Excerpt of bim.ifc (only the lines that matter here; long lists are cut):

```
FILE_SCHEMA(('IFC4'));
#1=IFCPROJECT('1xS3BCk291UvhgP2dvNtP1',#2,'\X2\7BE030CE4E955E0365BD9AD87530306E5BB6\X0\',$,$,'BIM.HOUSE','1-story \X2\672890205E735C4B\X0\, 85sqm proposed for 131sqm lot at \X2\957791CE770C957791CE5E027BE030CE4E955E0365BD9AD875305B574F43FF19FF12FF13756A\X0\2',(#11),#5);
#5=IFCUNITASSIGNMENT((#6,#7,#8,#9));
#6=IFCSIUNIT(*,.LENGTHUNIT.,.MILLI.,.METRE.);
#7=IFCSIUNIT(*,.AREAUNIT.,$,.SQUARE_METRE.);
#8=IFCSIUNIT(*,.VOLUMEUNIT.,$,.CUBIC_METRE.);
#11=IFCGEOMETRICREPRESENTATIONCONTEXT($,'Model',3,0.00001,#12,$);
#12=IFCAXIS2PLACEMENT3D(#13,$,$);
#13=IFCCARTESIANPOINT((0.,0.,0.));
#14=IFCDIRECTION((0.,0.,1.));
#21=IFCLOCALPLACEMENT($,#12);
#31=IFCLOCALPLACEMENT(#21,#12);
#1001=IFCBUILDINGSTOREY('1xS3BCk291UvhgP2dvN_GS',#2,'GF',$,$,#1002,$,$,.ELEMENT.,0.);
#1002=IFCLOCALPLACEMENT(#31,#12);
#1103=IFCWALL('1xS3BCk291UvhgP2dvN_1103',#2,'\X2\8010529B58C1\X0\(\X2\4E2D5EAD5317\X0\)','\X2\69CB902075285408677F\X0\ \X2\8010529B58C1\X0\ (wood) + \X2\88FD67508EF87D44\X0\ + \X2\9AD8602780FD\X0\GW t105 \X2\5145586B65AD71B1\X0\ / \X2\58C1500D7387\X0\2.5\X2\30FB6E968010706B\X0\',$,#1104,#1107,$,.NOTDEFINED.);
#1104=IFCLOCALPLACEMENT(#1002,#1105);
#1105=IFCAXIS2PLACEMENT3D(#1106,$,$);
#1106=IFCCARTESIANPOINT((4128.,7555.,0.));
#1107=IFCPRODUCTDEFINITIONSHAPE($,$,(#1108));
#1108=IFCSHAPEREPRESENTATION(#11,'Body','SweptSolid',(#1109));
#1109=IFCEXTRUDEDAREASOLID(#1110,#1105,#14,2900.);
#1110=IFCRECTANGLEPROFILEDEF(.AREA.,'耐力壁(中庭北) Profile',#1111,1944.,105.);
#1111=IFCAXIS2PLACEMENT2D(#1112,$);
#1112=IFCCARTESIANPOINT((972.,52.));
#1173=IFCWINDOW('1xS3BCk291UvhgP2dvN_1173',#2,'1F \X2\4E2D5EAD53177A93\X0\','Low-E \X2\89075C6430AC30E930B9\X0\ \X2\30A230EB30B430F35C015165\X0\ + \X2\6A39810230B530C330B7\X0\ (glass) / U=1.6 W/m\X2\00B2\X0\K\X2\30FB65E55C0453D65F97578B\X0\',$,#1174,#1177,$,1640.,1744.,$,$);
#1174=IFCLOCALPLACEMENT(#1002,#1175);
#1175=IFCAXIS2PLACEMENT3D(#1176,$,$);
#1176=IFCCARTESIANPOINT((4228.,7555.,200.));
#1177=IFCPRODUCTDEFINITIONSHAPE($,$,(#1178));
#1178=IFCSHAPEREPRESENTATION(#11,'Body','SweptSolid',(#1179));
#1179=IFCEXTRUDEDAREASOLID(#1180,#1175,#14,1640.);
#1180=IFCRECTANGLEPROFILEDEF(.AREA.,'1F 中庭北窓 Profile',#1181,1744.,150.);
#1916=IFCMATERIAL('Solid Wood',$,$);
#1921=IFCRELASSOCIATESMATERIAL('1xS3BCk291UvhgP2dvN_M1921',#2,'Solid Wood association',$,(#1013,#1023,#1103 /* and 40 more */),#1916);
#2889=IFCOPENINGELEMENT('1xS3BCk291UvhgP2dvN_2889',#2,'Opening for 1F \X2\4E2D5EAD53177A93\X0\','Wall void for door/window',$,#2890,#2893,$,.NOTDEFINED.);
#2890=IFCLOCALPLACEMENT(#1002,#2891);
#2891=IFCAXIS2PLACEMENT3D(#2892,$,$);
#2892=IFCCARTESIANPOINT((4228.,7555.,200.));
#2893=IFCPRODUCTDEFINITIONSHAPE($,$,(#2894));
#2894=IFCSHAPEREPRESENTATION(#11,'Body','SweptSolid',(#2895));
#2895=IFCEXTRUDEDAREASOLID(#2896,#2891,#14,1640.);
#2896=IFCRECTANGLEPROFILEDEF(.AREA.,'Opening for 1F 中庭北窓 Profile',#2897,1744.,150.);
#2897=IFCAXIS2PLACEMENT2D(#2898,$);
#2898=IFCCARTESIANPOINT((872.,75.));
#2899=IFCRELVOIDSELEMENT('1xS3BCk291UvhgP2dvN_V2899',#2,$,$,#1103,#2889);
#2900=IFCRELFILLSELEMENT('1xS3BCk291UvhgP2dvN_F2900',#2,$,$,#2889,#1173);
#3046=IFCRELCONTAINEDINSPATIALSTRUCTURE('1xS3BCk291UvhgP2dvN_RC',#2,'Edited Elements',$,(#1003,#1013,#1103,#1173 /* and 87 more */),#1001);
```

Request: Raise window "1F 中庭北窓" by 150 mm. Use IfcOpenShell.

```python
import numpy as np
import ifcopenshell
import ifcopenshell.api.geometry
import ifcopenshell.util.placement
import ifcopenshell.util.unit

model = ifcopenshell.open("bim.ifc")
unit_scale = ifcopenshell.util.unit.calculate_unit_scale(model)

window = model.by_guid("1xS3BCk291UvhgP2dvN_1173")
opening = window.FillsVoids[0].RelatingOpeningElement
dz = 0.15 / unit_scale

shift = np.array([0.0, 0.0, dz])
# The window is not placed relative to its opening, so move both.
for product in (opening, window):
    matrix = ifcopenshell.util.placement.get_local_placement(product.ObjectPlacement)
    matrix[:3, 3] += shift
    ifcopenshell.api.geometry.edit_object_placement(model, product=product, matrix=matrix, is_si=False)

print(f"moved by {dz * unit_scale:+.3f} m")

model.write("bim_edited.ifc")
```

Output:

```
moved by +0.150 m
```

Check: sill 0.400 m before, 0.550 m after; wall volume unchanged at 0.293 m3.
